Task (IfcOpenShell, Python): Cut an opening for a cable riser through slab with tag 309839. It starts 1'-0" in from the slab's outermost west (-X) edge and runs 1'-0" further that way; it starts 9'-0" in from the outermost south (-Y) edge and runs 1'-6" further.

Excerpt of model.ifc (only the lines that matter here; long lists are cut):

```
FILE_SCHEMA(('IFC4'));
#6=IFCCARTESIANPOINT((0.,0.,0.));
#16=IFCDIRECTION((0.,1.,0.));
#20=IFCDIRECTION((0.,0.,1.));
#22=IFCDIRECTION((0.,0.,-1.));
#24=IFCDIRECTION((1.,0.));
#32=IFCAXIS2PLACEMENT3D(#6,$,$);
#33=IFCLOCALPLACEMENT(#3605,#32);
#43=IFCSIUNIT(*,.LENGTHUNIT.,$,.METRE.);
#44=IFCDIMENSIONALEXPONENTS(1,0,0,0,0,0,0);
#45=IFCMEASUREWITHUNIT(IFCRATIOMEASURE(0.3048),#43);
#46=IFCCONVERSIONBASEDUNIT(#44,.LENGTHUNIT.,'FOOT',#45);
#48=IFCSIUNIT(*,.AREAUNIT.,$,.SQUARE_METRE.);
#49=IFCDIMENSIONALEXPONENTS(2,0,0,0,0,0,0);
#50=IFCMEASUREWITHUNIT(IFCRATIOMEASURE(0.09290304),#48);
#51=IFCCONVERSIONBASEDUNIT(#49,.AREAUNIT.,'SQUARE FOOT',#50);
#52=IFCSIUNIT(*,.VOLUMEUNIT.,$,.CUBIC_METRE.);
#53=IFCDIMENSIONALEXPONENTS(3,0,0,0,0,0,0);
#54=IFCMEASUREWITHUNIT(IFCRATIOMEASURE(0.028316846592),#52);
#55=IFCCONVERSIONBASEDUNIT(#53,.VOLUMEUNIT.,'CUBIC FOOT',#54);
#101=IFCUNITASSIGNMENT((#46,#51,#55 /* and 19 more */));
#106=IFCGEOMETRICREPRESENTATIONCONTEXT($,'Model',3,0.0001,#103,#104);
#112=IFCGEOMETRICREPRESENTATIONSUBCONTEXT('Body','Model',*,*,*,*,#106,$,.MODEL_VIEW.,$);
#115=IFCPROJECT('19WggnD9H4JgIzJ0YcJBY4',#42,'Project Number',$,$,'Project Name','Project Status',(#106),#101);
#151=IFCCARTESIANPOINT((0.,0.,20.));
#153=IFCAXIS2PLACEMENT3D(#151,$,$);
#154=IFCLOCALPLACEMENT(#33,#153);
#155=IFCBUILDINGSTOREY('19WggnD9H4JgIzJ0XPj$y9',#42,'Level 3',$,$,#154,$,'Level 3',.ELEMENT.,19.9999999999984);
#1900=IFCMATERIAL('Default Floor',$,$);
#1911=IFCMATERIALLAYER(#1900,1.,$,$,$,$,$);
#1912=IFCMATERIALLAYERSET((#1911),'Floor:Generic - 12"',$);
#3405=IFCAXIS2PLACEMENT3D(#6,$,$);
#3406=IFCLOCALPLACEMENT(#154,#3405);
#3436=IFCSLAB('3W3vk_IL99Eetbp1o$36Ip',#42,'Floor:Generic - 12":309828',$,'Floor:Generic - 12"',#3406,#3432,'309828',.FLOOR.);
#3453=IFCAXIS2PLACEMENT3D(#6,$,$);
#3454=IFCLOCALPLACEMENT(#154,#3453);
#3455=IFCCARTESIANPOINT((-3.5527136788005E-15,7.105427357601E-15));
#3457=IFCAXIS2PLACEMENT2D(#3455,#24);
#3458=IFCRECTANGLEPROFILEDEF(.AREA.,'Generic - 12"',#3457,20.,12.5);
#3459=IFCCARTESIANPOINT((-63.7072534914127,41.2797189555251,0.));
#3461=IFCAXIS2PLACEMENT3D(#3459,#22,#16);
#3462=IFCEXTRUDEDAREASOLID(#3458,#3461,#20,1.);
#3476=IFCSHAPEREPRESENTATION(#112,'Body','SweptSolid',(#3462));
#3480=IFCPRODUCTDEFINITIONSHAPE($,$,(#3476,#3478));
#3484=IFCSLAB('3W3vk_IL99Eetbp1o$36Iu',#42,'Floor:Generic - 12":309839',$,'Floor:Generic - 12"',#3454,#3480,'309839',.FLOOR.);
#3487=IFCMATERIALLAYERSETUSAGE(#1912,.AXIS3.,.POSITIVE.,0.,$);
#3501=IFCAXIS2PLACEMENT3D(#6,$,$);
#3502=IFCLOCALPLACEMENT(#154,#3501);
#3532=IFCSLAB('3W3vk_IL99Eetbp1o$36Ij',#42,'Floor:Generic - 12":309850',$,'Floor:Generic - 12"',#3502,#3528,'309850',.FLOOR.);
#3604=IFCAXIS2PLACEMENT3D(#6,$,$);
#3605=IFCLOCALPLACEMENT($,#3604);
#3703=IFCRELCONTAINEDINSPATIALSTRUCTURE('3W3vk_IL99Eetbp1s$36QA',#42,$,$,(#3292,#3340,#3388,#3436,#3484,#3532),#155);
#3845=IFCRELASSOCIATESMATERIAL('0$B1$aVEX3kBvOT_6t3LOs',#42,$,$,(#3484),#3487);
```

```python
import numpy as np
import ifcopenshell
import ifcopenshell.api.feature
import ifcopenshell.api.geometry
import ifcopenshell.api.root
import ifcopenshell.geom
import ifcopenshell.util.placement
import ifcopenshell.util.representation
import ifcopenshell.util.shape
import ifcopenshell.util.unit

model = ifcopenshell.open("model.ifc")
unit_scale = ifcopenshell.util.unit.calculate_unit_scale(model)
settings = ifcopenshell.geom.settings()


def volume(element):
    """Net volume in cubic metres, openings subtracted."""
    shape = ifcopenshell.geom.create_shape(settings, element)
    return ifcopenshell.util.shape.get_volume(shape.geometry)


slab = model.by_guid("3W3vk_IL99Eetbp1o$36Iu")
before = volume(slab)

# Extent in the slab's own axes, in metres. The edges named are its -X and -Y sides.
slab_shape = ifcopenshell.geom.create_shape(settings, slab)
vertices = ifcopenshell.util.shape.get_vertices(slab_shape.geometry)
x_min, y_min, bottom = vertices.min(axis=0)
top = vertices[:, 2].max()

opening = ifcopenshell.api.root.create_entity(model, ifc_class="IfcOpeningElement", name="Cable riser opening", predefined_type="OPENING")
context = ifcopenshell.util.representation.get_context(model, "Model", "Body", "MODEL_VIEW")
width, depth = 0.3048, 0.4572
outline = [(0.0, 0.0), (width, 0.0), (width, depth), (0.0, depth), (0.0, 0.0)]
# Overshoot both faces by 50 mm so the cut is clean.
shape = ifcopenshell.api.geometry.add_slab_representation(
    model, context=context, depth=top - bottom + 0.1, polyline=outline
)
ifcopenshell.api.geometry.assign_representation(model, product=opening, representation=shape)

matrix = ifcopenshell.util.placement.get_local_placement(slab.ObjectPlacement)
matrix[:, 3] = matrix @ np.append(np.array([x_min + 0.3048, y_min + 2.7432, bottom - 0.05]) / unit_scale, 1.0)
ifcopenshell.api.geometry.edit_object_placement(model, product=opening, matrix=matrix, is_si=False)
ifcopenshell.api.feature.add_feature(model, feature=opening, element=slab)

after = volume(slab)

print(f"slab volume {before:.3f} -> {after:.3f} m3")

model.write("model_rev.ifc")
```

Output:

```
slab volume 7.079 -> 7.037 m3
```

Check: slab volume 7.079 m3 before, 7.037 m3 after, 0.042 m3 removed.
